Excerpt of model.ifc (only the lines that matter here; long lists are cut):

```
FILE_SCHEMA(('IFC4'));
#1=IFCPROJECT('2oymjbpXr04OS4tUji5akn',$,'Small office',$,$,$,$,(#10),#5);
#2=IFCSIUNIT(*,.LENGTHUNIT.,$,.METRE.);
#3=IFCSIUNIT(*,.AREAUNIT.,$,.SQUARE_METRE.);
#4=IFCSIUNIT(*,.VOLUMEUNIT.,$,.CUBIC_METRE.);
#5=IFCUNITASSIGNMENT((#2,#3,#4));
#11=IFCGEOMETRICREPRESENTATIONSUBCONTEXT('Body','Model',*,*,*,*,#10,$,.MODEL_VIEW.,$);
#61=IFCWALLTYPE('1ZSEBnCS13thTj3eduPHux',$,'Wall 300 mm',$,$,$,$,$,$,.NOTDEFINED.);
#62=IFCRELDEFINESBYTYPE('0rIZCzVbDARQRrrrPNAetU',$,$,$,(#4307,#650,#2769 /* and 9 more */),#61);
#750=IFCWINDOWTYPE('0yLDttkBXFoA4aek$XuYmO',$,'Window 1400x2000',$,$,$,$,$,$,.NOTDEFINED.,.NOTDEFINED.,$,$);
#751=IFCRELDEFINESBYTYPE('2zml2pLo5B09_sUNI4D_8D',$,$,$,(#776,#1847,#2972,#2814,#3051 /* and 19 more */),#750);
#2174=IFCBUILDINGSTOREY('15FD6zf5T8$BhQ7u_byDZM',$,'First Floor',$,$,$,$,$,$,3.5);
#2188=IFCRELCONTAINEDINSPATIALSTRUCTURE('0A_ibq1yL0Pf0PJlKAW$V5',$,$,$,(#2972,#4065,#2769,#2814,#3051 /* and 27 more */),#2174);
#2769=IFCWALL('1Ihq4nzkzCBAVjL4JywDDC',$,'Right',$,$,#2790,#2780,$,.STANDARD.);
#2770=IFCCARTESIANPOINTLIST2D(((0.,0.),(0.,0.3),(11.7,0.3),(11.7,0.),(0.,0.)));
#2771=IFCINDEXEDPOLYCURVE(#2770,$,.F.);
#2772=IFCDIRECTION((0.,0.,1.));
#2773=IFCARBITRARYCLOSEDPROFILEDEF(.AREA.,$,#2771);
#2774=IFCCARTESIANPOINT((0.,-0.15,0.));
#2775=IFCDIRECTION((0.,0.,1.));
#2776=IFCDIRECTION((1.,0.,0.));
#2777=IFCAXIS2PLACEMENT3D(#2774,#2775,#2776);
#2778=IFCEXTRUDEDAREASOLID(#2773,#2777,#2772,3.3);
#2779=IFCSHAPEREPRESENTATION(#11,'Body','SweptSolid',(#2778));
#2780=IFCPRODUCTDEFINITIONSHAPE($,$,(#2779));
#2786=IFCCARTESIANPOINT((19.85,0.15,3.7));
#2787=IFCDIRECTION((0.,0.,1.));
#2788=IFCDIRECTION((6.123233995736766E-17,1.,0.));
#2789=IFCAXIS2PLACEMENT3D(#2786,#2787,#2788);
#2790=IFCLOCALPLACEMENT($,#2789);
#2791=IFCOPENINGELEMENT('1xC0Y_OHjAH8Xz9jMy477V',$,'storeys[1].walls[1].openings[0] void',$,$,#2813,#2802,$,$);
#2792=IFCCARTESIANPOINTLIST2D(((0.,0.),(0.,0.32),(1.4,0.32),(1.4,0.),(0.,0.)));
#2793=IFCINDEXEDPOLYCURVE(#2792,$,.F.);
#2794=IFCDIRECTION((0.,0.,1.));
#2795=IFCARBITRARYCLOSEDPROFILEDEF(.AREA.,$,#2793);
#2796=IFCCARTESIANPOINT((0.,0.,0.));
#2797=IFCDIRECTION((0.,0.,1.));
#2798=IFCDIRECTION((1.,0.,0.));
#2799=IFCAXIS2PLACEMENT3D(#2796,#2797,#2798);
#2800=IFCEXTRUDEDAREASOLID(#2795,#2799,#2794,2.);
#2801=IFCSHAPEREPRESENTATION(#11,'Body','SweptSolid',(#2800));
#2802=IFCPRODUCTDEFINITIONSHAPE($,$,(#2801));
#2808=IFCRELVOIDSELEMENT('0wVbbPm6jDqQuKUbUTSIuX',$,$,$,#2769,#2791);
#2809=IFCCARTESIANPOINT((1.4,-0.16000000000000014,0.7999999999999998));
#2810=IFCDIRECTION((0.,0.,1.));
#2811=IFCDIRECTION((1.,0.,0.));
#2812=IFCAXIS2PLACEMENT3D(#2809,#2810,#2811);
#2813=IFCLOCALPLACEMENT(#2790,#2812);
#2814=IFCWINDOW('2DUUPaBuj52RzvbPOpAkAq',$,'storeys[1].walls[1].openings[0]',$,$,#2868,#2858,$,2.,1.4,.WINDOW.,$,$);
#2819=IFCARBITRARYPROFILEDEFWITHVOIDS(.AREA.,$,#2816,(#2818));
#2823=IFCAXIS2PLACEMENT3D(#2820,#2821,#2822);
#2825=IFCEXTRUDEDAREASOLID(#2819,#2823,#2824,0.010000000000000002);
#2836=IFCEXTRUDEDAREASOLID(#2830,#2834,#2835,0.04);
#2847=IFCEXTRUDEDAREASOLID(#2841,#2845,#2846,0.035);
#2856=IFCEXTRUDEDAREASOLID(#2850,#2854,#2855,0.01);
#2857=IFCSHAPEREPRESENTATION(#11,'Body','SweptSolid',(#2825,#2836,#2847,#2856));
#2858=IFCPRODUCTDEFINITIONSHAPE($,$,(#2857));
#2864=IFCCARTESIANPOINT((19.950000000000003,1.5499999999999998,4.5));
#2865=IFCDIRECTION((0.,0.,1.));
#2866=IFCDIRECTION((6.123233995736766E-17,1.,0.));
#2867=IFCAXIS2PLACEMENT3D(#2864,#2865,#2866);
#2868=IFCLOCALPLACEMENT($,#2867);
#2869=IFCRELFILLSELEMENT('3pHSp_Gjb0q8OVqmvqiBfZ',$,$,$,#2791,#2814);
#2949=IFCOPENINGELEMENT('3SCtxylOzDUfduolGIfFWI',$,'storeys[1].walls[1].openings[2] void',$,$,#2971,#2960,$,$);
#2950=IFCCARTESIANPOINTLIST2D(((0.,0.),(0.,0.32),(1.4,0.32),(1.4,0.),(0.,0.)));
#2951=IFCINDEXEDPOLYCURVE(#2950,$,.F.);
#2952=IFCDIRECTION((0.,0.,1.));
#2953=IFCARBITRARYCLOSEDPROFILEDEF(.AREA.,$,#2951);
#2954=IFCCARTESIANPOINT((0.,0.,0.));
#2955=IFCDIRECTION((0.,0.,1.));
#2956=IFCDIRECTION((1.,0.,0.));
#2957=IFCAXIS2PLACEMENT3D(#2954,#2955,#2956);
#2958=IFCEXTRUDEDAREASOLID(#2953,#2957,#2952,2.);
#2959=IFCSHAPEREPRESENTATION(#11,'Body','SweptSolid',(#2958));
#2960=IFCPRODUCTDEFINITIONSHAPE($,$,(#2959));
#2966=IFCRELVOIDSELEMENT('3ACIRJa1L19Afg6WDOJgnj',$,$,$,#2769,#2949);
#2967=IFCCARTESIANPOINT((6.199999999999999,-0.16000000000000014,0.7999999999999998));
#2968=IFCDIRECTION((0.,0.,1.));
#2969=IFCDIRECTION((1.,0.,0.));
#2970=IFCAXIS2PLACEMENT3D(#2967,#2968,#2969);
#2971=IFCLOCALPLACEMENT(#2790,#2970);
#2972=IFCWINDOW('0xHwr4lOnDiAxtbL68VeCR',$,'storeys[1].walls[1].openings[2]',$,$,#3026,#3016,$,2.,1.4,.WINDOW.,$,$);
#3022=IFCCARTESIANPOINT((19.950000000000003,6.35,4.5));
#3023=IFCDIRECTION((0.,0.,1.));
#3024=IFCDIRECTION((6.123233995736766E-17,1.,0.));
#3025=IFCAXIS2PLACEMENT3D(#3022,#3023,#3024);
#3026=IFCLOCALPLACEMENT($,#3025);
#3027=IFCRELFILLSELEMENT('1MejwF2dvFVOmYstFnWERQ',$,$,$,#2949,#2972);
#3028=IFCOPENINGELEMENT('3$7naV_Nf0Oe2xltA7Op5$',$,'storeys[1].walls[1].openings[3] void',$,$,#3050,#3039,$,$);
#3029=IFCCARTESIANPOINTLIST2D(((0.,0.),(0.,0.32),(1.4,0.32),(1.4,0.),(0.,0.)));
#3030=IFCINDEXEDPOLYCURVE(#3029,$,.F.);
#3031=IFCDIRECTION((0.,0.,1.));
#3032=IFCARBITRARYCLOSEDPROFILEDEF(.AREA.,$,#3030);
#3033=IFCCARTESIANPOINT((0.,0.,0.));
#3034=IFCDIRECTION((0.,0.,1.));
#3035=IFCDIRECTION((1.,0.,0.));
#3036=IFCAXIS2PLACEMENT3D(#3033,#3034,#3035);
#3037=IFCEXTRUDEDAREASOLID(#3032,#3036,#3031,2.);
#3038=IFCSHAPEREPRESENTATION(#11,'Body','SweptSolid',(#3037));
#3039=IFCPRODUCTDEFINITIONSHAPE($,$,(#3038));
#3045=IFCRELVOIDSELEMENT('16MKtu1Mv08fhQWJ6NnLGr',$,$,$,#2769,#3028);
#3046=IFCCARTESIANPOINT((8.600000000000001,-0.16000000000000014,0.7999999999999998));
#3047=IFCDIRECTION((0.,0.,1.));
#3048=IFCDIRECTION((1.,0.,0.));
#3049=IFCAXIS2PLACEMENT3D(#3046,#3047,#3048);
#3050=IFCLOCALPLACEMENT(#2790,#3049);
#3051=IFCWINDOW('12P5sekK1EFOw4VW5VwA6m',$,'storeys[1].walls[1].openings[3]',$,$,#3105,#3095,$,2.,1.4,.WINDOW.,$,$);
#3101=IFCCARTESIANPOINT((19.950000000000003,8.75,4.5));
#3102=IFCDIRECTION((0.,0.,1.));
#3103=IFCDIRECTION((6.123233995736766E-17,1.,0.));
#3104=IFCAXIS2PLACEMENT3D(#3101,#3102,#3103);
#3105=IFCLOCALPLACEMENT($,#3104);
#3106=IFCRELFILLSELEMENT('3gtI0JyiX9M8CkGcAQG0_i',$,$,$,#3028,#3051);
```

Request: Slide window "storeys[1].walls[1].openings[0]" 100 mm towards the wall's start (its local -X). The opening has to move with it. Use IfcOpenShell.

```python
import ifcopenshell
import ifcopenshell.api.geometry
import ifcopenshell.util.placement

model = ifcopenshell.open("model.ifc")

window = model.by_guid("2DUUPaBuj52RzvbPOpAkAq")
opening = window.FillsVoids[0].RelatingOpeningElement
wall = opening.VoidsElements[0].RelatingBuildingElement

wall_matrix = ifcopenshell.util.placement.get_local_placement(wall.ObjectPlacement)
shift = wall_matrix[:3, 0] * -0.1
before = ifcopenshell.util.placement.get_local_placement(window.ObjectPlacement)[:3, 3].copy()

# The window is not placed relative to its opening, so move both.
for product in (opening, window):
    matrix = ifcopenshell.util.placement.get_local_placement(product.ObjectPlacement)
    matrix[:3, 3] += shift
    ifcopenshell.api.geometry.edit_object_placement(model, product=product, matrix=matrix, is_si=False)

after = ifcopenshell.util.placement.get_local_placement(window.ObjectPlacement)[:3, 3]
print("window moved by", (after - before).round(3) + 0.0)

model.write("model_v2.ifc")
```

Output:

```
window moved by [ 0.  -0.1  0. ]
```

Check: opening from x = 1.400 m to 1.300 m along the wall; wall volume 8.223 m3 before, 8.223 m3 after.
